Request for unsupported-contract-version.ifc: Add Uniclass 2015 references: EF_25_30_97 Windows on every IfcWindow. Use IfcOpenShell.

First a look at what the model holds.

```python
import ifcopenshell

model = ifcopenshell.open("unsupported-contract-version.ifc")
print(model.schema)
print("classifications:", [c.Name for c in model.by_type("IfcClassification")])
for ifc_class in ("IfcDoor", "IfcRoof", "IfcStair", "IfcWall", "IfcWindow"):
    print(ifc_class, len(model.by_type(ifc_class)))
```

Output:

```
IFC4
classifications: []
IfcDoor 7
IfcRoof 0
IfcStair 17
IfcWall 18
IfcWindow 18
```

```python
import ifcopenshell
import ifcopenshell.api.classification

model = ifcopenshell.open("unsupported-contract-version.ifc")

system = ifcopenshell.api.classification.add_classification(model, classification="Uniclass 2015")

codes = {
    "IfcWindow": ("EF_25_30_97", "Windows"),
}
for ifc_class, (code, name) in codes.items():
    products = model.by_type(ifc_class)
    ifcopenshell.api.classification.add_reference(
        model, products=products, classification=system, identification=code, name=name
    )
    print(code, len(products))

model.write("unsupported-contract-version-out.ifc")
```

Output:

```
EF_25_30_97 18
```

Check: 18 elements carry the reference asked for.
